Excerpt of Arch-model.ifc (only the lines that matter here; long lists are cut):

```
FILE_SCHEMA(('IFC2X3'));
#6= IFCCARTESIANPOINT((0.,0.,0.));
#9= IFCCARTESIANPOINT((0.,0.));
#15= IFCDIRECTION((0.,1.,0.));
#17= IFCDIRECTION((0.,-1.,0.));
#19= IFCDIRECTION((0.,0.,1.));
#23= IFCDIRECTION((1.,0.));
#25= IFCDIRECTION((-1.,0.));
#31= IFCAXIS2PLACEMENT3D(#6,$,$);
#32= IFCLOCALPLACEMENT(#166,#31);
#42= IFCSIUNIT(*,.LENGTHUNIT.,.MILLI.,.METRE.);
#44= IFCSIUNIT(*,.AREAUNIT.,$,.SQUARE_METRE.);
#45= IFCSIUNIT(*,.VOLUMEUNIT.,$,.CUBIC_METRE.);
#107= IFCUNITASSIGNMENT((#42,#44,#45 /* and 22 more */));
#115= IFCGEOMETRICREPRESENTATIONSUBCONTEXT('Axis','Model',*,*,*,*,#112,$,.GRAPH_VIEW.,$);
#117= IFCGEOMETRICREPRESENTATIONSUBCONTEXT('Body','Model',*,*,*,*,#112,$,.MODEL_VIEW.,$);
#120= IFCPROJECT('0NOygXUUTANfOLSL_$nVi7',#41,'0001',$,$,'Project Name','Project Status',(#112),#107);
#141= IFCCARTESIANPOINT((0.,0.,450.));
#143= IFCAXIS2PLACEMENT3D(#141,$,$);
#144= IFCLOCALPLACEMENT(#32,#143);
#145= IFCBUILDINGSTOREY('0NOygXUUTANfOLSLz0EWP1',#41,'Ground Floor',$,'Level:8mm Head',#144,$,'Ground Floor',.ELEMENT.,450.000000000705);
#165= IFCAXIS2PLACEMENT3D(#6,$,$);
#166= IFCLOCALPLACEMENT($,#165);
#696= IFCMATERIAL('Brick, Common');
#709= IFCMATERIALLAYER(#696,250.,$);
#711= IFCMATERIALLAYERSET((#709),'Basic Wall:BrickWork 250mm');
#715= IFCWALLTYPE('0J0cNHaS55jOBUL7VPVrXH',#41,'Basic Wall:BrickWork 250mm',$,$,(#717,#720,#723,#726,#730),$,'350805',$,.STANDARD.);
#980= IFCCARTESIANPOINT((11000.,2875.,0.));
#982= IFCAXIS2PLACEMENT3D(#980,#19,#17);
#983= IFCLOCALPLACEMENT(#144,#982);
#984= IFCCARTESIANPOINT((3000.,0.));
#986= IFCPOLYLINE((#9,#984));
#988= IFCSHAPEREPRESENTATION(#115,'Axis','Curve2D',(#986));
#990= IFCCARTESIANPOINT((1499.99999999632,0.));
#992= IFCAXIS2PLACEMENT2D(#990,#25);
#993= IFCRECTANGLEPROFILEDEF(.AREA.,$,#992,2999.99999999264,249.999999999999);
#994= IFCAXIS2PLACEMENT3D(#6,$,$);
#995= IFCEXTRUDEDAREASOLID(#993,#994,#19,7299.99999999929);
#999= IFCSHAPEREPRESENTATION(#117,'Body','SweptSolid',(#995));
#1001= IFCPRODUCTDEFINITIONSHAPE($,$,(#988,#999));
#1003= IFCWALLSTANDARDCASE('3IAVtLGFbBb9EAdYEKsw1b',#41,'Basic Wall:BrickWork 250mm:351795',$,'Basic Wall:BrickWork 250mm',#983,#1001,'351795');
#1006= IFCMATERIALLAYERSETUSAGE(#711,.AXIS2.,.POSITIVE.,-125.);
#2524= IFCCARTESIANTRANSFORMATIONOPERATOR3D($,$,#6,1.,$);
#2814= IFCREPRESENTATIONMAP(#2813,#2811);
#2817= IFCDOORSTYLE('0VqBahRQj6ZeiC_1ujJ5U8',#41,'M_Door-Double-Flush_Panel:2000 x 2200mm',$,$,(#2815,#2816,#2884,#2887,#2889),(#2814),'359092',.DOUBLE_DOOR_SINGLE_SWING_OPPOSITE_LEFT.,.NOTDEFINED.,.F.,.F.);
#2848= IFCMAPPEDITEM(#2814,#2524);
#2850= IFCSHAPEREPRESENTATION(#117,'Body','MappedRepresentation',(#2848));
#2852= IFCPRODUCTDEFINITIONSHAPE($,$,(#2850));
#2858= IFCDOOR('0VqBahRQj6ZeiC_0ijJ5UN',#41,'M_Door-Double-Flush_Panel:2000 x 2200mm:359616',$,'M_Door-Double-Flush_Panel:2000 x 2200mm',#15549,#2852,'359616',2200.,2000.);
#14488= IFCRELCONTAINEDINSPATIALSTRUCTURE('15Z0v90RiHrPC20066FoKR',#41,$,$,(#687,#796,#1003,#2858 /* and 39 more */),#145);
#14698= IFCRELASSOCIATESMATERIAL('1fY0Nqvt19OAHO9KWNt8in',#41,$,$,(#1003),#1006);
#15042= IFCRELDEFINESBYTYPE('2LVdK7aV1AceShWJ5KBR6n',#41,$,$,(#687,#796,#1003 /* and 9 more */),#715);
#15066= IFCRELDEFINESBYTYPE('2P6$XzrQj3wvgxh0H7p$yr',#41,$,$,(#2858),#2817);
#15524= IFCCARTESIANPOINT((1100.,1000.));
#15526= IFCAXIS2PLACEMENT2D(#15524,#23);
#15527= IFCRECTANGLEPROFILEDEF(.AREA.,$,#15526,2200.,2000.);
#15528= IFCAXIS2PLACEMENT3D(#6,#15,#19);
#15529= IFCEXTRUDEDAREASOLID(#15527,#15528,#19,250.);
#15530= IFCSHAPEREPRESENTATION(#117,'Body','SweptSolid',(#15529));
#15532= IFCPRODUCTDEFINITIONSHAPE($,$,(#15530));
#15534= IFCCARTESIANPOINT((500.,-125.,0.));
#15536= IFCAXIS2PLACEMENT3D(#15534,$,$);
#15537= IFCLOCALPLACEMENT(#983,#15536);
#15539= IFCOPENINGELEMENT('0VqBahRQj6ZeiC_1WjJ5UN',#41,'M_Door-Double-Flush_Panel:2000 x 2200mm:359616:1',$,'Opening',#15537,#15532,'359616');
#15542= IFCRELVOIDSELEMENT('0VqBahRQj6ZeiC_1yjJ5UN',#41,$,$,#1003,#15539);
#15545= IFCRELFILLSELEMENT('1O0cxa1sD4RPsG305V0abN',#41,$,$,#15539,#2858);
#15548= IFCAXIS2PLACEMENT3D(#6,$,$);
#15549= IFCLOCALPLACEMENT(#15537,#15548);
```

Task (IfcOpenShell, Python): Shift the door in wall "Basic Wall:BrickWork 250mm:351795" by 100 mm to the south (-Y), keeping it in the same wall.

```python
import ifcopenshell
import ifcopenshell.api.geometry
import ifcopenshell.util.placement
import ifcopenshell.util.unit

model = ifcopenshell.open("Arch-model.ifc")
unit_scale = ifcopenshell.util.unit.calculate_unit_scale(model)

door = model.by_guid("0VqBahRQj6ZeiC_0ijJ5UN")
opening = door.FillsVoids[0].RelatingOpeningElement
wall = opening.VoidsElements[0].RelatingBuildingElement

wall_matrix = ifcopenshell.util.placement.get_local_placement(wall.ObjectPlacement)
shift = wall_matrix[:3, 0] * 0.1 / unit_scale
before = ifcopenshell.util.placement.get_local_placement(door.ObjectPlacement)[:3, 3].copy()

# The door is placed relative to its opening, so it follows when the opening moves.
matrix = ifcopenshell.util.placement.get_local_placement(opening.ObjectPlacement)
matrix[:3, 3] += shift
ifcopenshell.api.geometry.edit_object_placement(
    model, product=opening, matrix=matrix, is_si=False, should_transform_children=True
)

after = ifcopenshell.util.placement.get_local_placement(door.ObjectPlacement)[:3, 3]
print("door moved by", (after - before).round(3) + 0.0)

model.write("Arch-model_rev.ifc")
```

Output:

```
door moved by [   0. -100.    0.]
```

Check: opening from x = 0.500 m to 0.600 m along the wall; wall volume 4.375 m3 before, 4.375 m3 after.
